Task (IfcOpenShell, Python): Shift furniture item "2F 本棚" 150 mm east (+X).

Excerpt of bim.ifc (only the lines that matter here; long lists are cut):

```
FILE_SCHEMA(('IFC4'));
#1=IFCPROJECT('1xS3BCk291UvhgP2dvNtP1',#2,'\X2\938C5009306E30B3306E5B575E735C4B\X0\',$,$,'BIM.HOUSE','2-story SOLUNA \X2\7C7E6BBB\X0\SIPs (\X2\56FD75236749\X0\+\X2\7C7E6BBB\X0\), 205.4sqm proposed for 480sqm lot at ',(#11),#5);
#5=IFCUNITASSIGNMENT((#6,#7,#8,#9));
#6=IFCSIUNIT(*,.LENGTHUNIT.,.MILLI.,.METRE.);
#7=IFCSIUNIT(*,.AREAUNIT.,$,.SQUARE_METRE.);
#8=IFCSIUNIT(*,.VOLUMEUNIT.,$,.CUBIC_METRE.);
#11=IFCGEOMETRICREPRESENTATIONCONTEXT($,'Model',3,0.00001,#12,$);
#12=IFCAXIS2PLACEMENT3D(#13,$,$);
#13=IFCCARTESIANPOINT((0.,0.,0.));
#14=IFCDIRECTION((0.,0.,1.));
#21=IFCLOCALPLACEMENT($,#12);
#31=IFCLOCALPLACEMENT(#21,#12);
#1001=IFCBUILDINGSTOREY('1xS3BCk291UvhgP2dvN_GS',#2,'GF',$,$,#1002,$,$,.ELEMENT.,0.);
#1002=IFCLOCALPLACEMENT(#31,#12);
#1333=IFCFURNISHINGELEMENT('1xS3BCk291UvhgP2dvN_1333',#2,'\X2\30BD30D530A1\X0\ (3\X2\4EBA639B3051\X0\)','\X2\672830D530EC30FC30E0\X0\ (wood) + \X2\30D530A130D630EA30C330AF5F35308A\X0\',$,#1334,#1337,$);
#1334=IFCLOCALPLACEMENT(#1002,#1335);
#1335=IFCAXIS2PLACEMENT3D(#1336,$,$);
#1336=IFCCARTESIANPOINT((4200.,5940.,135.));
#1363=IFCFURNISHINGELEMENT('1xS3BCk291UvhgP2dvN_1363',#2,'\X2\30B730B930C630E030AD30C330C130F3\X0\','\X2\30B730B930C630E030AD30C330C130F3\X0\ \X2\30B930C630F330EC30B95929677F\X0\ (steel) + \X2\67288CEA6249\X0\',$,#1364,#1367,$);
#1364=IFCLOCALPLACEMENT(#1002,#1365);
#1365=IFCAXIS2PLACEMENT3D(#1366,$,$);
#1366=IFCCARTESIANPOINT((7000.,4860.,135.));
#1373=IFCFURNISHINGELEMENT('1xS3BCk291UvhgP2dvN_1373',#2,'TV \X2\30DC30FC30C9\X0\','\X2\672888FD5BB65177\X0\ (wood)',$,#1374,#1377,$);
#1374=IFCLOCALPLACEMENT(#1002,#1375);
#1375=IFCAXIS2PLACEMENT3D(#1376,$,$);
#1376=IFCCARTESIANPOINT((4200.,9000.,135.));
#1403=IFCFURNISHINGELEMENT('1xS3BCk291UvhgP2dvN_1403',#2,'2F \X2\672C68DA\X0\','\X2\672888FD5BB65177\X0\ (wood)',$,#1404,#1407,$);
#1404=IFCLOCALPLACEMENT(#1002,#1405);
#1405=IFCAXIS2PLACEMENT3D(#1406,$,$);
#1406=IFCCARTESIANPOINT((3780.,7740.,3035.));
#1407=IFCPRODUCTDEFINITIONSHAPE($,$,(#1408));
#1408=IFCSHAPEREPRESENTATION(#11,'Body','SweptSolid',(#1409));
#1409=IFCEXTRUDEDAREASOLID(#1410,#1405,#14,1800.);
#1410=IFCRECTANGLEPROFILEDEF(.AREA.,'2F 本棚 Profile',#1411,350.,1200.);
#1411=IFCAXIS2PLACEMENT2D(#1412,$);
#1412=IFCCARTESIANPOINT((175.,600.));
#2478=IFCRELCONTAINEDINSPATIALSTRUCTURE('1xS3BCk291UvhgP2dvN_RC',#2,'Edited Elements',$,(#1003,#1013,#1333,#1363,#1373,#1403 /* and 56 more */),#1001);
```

```python
import ifcopenshell
import ifcopenshell.api.geometry
import ifcopenshell.util.placement

model = ifcopenshell.open("bim.ifc")

item = model.by_guid("1xS3BCk291UvhgP2dvN_1403")
matrix = ifcopenshell.util.placement.get_local_placement(item.ObjectPlacement)
matrix[0, 3] += 150.0
ifcopenshell.api.geometry.edit_object_placement(model, product=item, matrix=matrix, is_si=False)

print(ifcopenshell.util.placement.get_local_placement(item.ObjectPlacement).round(3) + 0.0)

model.write("bim_v2.ifc")
```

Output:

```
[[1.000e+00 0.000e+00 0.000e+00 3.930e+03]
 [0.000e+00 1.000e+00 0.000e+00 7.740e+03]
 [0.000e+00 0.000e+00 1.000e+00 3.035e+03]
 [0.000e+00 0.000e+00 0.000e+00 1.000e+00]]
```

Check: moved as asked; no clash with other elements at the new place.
